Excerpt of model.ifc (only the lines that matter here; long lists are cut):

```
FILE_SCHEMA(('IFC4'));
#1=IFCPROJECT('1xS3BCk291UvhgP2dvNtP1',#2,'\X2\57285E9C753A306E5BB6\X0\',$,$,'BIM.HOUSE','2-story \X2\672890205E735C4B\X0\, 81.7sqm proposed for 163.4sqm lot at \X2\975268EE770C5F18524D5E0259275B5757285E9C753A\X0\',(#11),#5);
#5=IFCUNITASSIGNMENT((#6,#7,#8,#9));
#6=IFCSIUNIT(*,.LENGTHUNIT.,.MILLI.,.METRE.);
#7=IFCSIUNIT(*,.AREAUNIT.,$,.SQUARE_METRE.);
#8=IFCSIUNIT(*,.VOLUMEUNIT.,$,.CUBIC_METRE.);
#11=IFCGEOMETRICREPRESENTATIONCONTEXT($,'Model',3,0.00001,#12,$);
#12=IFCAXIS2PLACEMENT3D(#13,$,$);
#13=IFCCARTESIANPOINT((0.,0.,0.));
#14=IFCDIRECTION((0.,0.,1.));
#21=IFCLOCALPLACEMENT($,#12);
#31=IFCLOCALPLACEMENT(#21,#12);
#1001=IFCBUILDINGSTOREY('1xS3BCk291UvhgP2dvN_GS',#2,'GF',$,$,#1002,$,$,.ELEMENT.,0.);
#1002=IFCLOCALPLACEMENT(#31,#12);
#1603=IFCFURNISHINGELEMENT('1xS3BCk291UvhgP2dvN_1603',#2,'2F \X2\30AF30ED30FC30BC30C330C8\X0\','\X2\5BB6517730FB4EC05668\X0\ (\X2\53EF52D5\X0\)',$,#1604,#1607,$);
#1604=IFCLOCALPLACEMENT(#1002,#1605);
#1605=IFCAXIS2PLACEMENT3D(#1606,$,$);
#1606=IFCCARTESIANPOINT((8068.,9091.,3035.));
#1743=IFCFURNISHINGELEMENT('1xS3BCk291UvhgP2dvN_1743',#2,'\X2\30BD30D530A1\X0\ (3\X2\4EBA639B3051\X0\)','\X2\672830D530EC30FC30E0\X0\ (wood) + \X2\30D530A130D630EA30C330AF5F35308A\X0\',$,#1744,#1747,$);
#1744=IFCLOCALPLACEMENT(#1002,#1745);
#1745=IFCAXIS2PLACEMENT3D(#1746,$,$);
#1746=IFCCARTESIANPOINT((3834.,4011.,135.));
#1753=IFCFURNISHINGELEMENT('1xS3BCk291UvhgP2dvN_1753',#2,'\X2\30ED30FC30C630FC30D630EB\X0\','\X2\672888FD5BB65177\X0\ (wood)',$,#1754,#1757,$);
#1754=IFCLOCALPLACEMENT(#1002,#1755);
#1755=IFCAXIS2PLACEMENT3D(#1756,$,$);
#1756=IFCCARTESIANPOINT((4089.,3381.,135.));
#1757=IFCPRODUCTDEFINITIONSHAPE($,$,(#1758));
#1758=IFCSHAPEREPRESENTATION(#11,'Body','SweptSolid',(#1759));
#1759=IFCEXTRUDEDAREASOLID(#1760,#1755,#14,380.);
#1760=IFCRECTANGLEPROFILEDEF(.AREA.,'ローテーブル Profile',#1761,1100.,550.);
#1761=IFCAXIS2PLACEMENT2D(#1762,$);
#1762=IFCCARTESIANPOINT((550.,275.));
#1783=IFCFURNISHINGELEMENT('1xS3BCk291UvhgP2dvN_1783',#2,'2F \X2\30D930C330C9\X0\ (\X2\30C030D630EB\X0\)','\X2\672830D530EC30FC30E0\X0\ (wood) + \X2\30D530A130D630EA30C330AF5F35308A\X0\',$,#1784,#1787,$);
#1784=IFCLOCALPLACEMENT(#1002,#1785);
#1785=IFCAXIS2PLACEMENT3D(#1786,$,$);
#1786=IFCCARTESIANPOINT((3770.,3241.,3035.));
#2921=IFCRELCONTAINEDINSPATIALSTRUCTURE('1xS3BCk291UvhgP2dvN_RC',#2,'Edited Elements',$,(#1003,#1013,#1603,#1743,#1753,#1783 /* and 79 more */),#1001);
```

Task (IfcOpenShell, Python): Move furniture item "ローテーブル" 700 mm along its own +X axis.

```python
import ifcopenshell
import ifcopenshell.api.geometry
import ifcopenshell.util.placement
import ifcopenshell.util.unit

model = ifcopenshell.open("model.ifc")
unit_scale = ifcopenshell.util.unit.calculate_unit_scale(model)

item = model.by_guid("1xS3BCk291UvhgP2dvN_1753")
matrix = ifcopenshell.util.placement.get_local_placement(item.ObjectPlacement)
matrix[:3, 3] += matrix[:3, 0] * 0.7 / unit_scale
ifcopenshell.api.geometry.edit_object_placement(model, product=item, matrix=matrix, is_si=False)

print(ifcopenshell.util.placement.get_local_placement(item.ObjectPlacement).round(3) + 0.0)

model.write("model_v2.ifc")
```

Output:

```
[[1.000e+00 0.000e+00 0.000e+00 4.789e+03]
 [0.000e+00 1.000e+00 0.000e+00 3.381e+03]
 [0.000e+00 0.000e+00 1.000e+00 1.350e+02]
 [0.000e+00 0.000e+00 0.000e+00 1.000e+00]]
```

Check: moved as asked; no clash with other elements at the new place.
